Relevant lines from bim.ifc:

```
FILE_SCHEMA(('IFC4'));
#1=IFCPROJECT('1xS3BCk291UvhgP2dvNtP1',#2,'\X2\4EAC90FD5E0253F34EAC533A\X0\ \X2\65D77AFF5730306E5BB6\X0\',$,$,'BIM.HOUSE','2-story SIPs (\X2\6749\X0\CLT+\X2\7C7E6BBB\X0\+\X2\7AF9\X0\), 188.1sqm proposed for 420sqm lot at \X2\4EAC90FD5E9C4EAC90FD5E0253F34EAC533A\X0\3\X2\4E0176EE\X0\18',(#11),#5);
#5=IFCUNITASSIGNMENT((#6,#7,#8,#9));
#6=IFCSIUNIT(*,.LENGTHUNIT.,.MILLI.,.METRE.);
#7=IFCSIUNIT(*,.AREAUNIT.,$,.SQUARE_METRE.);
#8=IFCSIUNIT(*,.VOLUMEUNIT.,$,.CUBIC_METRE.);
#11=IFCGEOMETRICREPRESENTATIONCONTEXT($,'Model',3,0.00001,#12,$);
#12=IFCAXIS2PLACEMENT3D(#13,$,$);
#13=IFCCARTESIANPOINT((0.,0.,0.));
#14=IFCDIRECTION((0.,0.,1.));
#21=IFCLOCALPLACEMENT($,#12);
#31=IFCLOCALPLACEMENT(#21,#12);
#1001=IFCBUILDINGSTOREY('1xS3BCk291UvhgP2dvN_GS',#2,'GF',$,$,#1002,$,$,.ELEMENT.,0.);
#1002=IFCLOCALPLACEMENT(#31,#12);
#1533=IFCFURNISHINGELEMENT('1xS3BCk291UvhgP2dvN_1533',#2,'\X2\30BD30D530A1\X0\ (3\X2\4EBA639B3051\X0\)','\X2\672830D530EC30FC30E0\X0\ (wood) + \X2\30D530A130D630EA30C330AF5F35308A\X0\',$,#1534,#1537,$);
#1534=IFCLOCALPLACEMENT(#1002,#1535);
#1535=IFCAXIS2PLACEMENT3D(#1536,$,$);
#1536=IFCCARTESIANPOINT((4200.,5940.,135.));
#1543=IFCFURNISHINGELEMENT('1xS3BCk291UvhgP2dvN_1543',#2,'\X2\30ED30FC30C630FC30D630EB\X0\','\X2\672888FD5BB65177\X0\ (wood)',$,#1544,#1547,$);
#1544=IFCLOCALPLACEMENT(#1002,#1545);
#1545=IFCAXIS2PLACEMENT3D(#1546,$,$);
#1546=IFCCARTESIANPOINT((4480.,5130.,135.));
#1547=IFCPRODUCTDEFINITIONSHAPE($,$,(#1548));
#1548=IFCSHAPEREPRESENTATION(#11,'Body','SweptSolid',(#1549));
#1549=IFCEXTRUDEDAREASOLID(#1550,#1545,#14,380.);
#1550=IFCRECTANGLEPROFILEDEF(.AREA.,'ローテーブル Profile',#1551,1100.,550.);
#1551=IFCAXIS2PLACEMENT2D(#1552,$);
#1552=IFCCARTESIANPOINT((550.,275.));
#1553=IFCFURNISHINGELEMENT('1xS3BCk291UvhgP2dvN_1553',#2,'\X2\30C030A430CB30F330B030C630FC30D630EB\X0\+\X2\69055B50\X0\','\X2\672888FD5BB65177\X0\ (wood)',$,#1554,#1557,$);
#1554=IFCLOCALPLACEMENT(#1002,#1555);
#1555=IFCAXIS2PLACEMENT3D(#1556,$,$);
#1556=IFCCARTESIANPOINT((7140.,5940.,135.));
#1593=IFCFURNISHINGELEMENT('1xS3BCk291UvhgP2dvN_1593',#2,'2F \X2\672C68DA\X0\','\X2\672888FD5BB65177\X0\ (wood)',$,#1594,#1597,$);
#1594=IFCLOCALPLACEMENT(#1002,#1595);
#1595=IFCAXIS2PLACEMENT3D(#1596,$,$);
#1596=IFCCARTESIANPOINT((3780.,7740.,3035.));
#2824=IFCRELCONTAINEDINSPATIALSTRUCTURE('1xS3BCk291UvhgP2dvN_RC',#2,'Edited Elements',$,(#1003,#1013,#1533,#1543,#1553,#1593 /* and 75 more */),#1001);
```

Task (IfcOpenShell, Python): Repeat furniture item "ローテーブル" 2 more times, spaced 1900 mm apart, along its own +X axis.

```python
import ifcopenshell
import ifcopenshell.api.geometry
import ifcopenshell.api.root
import ifcopenshell.util.element
import ifcopenshell.util.placement

model = ifcopenshell.open("bim.ifc")


def reuse_history(source, copy):
    """copy_class also copies each property set's owner history, people and application; keep the originals."""
    for rel in copy.IsDefinedBy:
        if rel.is_a("IfcRelDefinesByProperties") and (history := rel.RelatingPropertyDefinition.OwnerHistory):
            rel.RelatingPropertyDefinition.OwnerHistory = source.OwnerHistory
            ifcopenshell.util.element.remove_deep2(model, history)


source = model.by_id(1543)
base = ifcopenshell.util.placement.get_local_placement(source.ObjectPlacement)
step = base[:3, 0] * 1900.0

for i in range(1, 3):
    copy = ifcopenshell.api.root.copy_class(model, product=source)
    copy.Representation = ifcopenshell.util.element.copy_deep(
        model, source.Representation, exclude=["IfcGeometricRepresentationContext", "IfcRepresentationMap"]
    )
    reuse_history(source, copy)
    matrix = base.copy()
    matrix[:3, 3] += i * step
    print("added at", matrix[:3, 3].round(3) + 0.0)
    ifcopenshell.api.geometry.edit_object_placement(model, product=copy, matrix=matrix, is_si=False)

model.write("bim_v2.ifc")
```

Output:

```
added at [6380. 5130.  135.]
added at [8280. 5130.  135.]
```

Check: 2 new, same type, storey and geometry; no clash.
